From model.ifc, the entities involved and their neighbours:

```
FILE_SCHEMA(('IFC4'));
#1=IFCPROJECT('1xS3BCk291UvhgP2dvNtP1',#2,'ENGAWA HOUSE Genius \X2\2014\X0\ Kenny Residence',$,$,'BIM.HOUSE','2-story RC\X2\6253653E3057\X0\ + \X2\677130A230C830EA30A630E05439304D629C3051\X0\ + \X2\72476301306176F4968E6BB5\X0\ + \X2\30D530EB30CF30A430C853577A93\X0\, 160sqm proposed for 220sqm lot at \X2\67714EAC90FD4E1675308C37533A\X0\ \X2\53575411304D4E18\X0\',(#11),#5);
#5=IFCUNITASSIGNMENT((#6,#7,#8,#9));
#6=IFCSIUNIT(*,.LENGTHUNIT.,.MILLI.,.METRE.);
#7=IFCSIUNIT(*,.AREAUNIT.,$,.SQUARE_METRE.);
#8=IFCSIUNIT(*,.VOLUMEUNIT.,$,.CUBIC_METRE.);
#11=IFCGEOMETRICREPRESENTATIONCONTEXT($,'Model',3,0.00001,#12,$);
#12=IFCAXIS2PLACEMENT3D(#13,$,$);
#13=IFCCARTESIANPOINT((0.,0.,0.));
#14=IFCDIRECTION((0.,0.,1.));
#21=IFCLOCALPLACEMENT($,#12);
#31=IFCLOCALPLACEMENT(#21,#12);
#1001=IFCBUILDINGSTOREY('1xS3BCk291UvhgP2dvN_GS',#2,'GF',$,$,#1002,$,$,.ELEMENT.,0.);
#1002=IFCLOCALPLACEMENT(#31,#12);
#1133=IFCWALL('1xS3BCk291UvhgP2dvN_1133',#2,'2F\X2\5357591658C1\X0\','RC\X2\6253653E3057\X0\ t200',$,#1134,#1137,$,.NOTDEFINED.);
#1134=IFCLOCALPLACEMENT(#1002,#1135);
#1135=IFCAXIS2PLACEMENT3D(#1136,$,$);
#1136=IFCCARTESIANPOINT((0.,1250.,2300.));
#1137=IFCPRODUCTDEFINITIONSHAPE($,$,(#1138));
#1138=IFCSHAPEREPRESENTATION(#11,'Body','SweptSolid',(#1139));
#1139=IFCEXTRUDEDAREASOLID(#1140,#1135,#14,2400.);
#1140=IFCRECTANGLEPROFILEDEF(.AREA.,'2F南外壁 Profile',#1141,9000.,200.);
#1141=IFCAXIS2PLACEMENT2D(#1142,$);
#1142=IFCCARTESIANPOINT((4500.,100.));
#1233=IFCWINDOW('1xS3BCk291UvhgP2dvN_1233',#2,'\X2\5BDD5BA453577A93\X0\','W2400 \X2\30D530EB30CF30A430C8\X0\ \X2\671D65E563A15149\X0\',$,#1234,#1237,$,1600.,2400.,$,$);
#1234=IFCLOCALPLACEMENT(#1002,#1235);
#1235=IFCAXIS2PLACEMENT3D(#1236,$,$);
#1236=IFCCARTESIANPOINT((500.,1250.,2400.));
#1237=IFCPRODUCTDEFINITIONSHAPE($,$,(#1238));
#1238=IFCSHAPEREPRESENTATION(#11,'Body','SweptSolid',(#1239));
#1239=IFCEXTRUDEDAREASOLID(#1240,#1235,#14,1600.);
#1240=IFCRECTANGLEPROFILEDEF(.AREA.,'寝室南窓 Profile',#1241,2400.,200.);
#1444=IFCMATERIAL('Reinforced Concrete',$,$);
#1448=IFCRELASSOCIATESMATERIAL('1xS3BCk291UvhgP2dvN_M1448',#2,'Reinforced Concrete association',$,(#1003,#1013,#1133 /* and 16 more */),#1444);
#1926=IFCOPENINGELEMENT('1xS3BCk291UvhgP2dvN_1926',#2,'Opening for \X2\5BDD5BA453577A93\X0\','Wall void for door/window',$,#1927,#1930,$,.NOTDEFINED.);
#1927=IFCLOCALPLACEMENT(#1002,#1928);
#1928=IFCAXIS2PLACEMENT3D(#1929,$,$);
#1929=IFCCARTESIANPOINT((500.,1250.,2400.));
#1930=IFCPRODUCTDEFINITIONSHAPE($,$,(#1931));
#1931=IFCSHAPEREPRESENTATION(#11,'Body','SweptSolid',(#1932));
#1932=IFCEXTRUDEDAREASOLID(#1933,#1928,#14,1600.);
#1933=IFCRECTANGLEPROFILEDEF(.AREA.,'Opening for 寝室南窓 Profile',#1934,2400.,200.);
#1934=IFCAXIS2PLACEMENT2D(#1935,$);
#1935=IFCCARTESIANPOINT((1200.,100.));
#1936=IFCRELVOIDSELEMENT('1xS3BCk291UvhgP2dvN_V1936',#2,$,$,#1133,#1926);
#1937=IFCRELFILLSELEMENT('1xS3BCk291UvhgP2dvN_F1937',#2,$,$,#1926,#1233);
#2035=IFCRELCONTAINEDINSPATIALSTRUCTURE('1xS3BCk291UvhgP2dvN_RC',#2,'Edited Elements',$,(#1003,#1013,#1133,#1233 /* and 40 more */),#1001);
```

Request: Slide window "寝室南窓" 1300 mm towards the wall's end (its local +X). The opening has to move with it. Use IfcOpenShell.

```python
import ifcopenshell
import ifcopenshell.api.geometry
import ifcopenshell.util.placement

model = ifcopenshell.open("model.ifc")

window = model.by_id(1233)
opening = window.FillsVoids[0].RelatingOpeningElement
wall = opening.VoidsElements[0].RelatingBuildingElement

wall_matrix = ifcopenshell.util.placement.get_local_placement(wall.ObjectPlacement)
shift = wall_matrix[:3, 0] * 1300.0
before = ifcopenshell.util.placement.get_local_placement(window.ObjectPlacement)[:3, 3].copy()

# The window is not placed relative to its opening, so move both.
for product in (opening, window):
    matrix = ifcopenshell.util.placement.get_local_placement(product.ObjectPlacement)
    matrix[:3, 3] += shift
    ifcopenshell.api.geometry.edit_object_placement(model, product=product, matrix=matrix, is_si=False)

after = ifcopenshell.util.placement.get_local_placement(window.ObjectPlacement)[:3, 3]
print("window moved by", (after - before).round(3) + 0.0)

model.write("model-out.ifc")
```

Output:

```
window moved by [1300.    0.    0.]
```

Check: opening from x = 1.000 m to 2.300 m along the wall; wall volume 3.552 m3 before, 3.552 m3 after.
